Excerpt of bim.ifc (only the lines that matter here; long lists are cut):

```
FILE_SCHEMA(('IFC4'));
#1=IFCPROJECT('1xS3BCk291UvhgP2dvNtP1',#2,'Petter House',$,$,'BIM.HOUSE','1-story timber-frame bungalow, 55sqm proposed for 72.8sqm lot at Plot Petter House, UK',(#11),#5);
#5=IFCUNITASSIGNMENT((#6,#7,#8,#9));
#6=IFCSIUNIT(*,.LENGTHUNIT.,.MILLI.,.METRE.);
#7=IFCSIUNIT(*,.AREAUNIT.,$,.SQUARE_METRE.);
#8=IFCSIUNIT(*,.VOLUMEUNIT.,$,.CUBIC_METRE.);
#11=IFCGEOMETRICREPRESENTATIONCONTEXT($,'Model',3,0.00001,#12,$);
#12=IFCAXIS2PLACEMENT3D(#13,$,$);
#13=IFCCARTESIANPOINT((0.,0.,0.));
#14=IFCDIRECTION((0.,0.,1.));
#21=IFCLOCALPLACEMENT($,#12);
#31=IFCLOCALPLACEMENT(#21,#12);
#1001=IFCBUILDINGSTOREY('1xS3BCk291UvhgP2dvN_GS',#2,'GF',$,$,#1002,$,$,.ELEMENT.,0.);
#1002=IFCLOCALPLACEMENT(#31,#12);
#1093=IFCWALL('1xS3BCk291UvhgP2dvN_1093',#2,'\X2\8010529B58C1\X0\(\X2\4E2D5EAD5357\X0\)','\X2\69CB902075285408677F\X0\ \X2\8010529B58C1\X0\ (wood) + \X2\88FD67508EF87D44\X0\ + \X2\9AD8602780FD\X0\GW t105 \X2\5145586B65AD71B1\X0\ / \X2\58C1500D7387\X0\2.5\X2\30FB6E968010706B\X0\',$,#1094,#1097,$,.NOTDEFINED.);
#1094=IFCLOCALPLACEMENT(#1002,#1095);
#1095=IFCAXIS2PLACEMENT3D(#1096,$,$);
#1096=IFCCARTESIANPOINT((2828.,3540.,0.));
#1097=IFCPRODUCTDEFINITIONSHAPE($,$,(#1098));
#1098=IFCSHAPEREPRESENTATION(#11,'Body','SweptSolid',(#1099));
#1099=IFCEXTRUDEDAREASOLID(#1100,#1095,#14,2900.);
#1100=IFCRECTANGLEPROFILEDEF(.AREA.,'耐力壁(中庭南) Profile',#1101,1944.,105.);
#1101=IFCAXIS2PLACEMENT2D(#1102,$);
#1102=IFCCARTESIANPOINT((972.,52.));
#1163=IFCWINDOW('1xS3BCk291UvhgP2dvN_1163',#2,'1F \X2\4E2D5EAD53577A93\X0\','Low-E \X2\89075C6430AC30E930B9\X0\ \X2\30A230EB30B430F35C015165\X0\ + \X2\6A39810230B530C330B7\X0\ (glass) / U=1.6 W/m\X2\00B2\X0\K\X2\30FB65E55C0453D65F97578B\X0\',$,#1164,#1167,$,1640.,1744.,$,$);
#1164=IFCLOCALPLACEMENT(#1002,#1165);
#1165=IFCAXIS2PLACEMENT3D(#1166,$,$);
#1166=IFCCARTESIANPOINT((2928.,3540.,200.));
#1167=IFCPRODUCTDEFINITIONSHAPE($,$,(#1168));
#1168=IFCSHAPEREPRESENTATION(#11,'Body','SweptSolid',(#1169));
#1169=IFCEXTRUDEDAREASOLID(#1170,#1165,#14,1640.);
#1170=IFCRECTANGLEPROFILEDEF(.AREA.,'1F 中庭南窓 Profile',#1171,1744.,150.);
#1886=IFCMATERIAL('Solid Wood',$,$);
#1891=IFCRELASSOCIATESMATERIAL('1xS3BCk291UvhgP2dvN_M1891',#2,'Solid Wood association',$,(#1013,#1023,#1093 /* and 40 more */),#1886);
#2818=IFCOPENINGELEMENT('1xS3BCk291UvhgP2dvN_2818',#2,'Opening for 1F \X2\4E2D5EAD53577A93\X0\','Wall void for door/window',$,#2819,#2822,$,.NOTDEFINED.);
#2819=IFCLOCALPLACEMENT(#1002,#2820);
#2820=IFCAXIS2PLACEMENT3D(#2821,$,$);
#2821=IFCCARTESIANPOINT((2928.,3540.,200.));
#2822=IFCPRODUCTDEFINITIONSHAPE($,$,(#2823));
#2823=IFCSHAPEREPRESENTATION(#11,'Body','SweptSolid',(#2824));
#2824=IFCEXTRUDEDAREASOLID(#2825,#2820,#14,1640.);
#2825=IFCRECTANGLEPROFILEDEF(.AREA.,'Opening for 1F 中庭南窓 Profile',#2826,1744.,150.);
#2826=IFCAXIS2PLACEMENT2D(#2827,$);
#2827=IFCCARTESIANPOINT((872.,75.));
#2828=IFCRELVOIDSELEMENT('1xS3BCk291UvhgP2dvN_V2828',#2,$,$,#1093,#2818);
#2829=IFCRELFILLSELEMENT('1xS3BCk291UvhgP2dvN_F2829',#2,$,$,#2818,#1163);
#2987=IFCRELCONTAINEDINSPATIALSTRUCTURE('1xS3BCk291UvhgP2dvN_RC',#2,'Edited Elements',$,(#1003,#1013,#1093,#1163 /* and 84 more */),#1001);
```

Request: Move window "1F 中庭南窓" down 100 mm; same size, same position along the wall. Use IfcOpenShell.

```python
import numpy as np
import ifcopenshell
import ifcopenshell.api.geometry
import ifcopenshell.util.placement
import ifcopenshell.util.unit

model = ifcopenshell.open("bim.ifc")
unit_scale = ifcopenshell.util.unit.calculate_unit_scale(model)

window = model.by_id(1163)
opening = window.FillsVoids[0].RelatingOpeningElement
dz = -0.1 / unit_scale

shift = np.array([0.0, 0.0, dz])
# The window is not placed relative to its opening, so move both.
for product in (opening, window):
    matrix = ifcopenshell.util.placement.get_local_placement(product.ObjectPlacement)
    matrix[:3, 3] += shift
    ifcopenshell.api.geometry.edit_object_placement(model, product=product, matrix=matrix, is_si=False)

print(f"moved by {dz * unit_scale:+.3f} m")

model.write("bim_updated.ifc")
```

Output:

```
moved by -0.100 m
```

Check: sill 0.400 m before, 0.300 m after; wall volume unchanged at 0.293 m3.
